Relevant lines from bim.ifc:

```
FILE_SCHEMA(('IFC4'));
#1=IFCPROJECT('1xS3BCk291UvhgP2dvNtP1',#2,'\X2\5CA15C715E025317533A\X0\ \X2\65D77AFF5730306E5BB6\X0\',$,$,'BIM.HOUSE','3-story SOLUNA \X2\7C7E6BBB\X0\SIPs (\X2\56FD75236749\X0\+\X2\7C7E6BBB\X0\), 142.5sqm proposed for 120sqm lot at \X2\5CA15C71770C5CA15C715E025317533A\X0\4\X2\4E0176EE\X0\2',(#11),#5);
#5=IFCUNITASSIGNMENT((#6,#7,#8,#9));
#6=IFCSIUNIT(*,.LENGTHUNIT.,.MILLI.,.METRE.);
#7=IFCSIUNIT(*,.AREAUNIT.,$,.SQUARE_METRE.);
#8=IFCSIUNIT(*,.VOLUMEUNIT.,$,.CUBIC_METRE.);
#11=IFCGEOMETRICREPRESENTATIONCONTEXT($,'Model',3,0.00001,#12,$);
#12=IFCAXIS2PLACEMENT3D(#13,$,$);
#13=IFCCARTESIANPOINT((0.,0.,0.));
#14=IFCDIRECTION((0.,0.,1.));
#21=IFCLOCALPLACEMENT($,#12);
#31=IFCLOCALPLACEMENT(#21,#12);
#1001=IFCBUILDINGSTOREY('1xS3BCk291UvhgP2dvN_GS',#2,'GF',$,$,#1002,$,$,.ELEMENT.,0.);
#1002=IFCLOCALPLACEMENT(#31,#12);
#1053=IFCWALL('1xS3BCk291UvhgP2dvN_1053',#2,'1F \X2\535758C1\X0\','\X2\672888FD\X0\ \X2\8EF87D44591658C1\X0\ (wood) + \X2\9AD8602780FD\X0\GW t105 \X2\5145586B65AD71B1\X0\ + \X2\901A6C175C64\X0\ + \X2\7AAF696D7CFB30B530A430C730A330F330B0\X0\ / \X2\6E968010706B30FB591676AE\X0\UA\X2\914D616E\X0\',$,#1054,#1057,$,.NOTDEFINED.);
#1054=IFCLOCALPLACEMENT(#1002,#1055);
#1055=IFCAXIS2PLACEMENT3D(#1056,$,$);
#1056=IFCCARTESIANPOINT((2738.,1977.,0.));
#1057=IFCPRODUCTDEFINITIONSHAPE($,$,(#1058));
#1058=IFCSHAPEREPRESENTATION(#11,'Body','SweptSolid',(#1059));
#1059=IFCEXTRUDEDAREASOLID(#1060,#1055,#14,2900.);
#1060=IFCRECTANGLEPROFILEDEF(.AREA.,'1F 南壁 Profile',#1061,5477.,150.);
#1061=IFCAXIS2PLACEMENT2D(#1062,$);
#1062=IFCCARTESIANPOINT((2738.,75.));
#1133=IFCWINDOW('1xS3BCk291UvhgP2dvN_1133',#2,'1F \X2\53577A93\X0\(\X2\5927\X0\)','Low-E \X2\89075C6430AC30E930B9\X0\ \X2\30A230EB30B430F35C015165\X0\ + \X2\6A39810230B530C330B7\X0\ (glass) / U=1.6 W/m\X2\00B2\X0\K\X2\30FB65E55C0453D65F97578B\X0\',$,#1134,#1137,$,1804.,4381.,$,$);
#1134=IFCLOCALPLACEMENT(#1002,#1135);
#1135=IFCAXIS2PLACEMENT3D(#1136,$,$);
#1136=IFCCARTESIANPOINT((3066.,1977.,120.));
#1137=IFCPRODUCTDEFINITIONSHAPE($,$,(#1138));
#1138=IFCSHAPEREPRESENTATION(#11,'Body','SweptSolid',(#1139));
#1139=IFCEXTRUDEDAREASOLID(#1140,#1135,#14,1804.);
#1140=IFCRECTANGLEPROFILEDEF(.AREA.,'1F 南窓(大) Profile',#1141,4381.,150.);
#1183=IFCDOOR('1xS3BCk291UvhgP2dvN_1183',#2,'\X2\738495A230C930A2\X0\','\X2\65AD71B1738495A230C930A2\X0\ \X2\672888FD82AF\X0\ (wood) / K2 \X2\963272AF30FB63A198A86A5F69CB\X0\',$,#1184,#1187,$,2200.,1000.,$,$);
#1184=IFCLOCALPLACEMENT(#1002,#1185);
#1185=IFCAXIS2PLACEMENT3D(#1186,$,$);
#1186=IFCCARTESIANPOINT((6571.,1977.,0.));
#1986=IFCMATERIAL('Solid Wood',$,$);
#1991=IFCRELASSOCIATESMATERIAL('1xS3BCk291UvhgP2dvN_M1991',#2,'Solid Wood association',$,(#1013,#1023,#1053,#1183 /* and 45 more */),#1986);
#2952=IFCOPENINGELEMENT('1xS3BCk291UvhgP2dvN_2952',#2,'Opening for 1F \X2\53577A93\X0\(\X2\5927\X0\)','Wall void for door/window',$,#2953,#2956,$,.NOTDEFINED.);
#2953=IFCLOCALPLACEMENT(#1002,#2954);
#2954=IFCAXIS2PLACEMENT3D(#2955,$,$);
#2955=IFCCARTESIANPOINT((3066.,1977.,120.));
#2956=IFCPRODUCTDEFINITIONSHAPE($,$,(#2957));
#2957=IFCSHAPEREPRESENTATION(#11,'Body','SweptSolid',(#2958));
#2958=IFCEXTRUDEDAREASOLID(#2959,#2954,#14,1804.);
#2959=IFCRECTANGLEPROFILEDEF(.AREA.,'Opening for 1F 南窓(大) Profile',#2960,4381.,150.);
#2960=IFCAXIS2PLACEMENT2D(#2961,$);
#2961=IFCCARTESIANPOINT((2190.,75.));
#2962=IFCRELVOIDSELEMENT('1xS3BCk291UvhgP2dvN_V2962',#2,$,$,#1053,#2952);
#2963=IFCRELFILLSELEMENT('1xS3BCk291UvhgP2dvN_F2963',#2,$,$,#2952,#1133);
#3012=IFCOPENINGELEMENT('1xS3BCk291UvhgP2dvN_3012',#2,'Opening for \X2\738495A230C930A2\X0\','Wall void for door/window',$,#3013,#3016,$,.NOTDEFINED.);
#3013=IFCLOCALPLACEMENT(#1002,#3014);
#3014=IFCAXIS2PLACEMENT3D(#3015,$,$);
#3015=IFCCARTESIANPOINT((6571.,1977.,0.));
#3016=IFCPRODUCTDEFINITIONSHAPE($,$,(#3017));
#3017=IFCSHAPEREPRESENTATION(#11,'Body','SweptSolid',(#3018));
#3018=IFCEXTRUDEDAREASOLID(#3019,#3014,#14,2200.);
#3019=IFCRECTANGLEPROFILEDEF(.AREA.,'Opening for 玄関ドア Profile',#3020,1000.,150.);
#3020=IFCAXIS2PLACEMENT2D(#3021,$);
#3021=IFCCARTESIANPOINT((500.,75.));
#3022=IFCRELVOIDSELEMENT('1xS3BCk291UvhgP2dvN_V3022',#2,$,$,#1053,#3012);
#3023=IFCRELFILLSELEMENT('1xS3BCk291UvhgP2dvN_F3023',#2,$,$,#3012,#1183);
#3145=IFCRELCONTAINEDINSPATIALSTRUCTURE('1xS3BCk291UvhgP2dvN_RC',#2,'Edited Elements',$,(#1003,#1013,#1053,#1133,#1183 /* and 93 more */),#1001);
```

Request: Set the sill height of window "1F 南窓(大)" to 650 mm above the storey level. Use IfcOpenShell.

```python
import numpy as np
import ifcopenshell
import ifcopenshell.api.geometry
import ifcopenshell.geom
import ifcopenshell.util.element
import ifcopenshell.util.placement
import ifcopenshell.util.shape
import ifcopenshell.util.unit

model = ifcopenshell.open("bim.ifc")
unit_scale = ifcopenshell.util.unit.calculate_unit_scale(model)

window = model.by_id(1133)
opening = window.FillsVoids[0].RelatingOpeningElement
storey = ifcopenshell.util.element.get_container(window, ifc_class="IfcBuildingStorey")
level = ifcopenshell.util.placement.get_local_placement(storey.ObjectPlacement)[2, 3]

# The opening's origin need not be at the sill, so measure its lowest point.
shape = ifcopenshell.geom.create_shape(ifcopenshell.geom.settings(), opening)
bottom = ifcopenshell.util.shape.get_shape_bottom_elevation(shape, shape.geometry) / unit_scale
dz = level + 650.0 - bottom

shift = np.array([0.0, 0.0, dz])
# The window is not placed relative to its opening, so move both.
for product in (opening, window):
    matrix = ifcopenshell.util.placement.get_local_placement(product.ObjectPlacement)
    matrix[:3, 3] += shift
    ifcopenshell.api.geometry.edit_object_placement(model, product=product, matrix=matrix, is_si=False)

print(f"moved by {dz * unit_scale:+.3f} m")

model.write("bim_rev.ifc")
```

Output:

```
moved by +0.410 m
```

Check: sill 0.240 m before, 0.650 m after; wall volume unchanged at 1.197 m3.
